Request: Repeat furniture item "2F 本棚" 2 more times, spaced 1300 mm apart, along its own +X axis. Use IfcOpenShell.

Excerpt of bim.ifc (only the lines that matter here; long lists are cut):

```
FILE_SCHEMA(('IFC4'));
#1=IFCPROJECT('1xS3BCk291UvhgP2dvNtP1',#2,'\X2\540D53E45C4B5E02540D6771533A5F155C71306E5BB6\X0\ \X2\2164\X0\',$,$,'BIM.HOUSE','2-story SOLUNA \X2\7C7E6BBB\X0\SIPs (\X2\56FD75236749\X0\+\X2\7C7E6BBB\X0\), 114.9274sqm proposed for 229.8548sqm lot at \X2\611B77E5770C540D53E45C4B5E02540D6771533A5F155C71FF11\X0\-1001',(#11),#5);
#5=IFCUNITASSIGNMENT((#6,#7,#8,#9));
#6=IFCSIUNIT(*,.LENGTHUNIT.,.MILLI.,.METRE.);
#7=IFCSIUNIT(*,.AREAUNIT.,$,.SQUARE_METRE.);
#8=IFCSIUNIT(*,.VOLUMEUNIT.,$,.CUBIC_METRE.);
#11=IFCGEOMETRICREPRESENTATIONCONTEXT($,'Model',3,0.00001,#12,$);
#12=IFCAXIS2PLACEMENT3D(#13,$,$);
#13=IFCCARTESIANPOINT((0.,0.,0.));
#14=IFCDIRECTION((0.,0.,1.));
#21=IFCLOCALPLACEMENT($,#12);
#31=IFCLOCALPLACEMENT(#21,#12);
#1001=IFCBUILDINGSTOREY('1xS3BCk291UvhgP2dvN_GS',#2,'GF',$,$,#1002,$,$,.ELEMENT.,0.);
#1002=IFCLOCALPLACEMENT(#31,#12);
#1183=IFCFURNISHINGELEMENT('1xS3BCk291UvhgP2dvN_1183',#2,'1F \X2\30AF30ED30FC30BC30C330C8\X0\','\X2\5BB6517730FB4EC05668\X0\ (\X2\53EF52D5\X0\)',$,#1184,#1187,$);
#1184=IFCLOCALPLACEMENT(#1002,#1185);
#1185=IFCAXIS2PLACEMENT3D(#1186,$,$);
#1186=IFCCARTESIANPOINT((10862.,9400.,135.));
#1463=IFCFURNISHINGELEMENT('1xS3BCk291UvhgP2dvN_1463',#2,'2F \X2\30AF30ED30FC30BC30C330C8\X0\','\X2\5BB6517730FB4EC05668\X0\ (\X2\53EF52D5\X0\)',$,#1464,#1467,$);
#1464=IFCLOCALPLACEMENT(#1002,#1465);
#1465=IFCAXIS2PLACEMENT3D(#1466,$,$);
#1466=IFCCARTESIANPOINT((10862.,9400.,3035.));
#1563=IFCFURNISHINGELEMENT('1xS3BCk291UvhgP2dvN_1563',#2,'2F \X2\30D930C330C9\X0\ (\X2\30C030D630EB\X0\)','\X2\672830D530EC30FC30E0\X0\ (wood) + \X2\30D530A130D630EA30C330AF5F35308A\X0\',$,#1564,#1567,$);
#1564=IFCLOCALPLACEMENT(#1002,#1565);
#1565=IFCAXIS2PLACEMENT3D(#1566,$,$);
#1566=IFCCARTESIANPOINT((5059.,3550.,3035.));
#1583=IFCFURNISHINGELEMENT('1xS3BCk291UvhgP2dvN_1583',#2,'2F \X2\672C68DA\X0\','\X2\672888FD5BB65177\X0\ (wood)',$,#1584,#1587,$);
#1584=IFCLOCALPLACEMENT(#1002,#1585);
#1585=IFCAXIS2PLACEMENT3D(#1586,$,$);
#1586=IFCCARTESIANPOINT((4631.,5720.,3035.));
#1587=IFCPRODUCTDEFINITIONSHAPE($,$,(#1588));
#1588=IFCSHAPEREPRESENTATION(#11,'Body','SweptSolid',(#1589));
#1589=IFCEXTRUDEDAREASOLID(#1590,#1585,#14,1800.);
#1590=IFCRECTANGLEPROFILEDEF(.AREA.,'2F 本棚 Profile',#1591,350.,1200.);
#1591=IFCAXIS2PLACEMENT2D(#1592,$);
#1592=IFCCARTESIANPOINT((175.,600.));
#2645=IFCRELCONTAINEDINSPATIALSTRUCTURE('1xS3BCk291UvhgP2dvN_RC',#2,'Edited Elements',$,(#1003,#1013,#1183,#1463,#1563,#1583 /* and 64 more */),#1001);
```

```python
import ifcopenshell
import ifcopenshell.api.geometry
import ifcopenshell.api.root
import ifcopenshell.util.element
import ifcopenshell.util.placement

model = ifcopenshell.open("bim.ifc")


def reuse_history(source, copy):
    """copy_class also copies each property set's owner history, people and application; keep the originals."""
    for rel in copy.IsDefinedBy:
        if rel.is_a("IfcRelDefinesByProperties") and (history := rel.RelatingPropertyDefinition.OwnerHistory):
            rel.RelatingPropertyDefinition.OwnerHistory = source.OwnerHistory
            ifcopenshell.util.element.remove_deep2(model, history)


source = model.by_guid("1xS3BCk291UvhgP2dvN_1583")
base = ifcopenshell.util.placement.get_local_placement(source.ObjectPlacement)
step = base[:3, 0] * 1300.0

for i in range(1, 3):
    copy = ifcopenshell.api.root.copy_class(model, product=source)
    copy.Representation = ifcopenshell.util.element.copy_deep(
        model, source.Representation, exclude=["IfcGeometricRepresentationContext", "IfcRepresentationMap"]
    )
    reuse_history(source, copy)
    matrix = base.copy()
    matrix[:3, 3] += i * step
    print("added at", matrix[:3, 3].round(3) + 0.0)
    ifcopenshell.api.geometry.edit_object_placement(model, product=copy, matrix=matrix, is_si=False)

model.write("bim_updated.ifc")
```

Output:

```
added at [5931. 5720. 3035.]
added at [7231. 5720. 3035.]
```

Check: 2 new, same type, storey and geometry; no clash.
